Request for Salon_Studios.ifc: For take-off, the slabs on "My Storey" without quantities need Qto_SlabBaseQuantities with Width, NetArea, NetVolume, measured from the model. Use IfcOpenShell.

First a look at what the model holds.

```python
import ifcopenshell
import ifcopenshell.util.element
import ifcopenshell.util.unit

model = ifcopenshell.open("Salon_Studios.ifc")
print(model.schema)
for unit_type in ("LENGTHUNIT", "AREAUNIT", "VOLUMEUNIT"):
    print(unit_type, ifcopenshell.util.unit.calculate_unit_scale(model, unit_type))
storey = next(s for s in model.by_type("IfcBuildingStorey") if s.Name == "My Storey")
slabs = [e for e in ifcopenshell.util.element.get_decomposition(storey) if e.is_a("IfcSlab")]
for e in sorted(slabs, key=lambda e: e.id()):
    print(e.id(), e.is_a(), e.Name, list(ifcopenshell.util.element.get_psets(e, qtos_only=True)), sep=" | ")
```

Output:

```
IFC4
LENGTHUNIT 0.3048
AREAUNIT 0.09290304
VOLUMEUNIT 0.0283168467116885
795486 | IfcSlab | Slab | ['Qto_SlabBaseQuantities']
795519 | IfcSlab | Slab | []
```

```python
import ifcopenshell
import ifcopenshell.api.pset
import ifcopenshell.geom
import ifcopenshell.util.element
import ifcopenshell.util.shape
import ifcopenshell.util.unit

model = ifcopenshell.open("Salon_Studios.ifc")
unit_scale = ifcopenshell.util.unit.calculate_unit_scale(model)
area_scale = ifcopenshell.util.unit.calculate_unit_scale(model, "AREAUNIT")
volume_scale = ifcopenshell.util.unit.calculate_unit_scale(model, "VOLUMEUNIT")
settings = ifcopenshell.geom.settings()

storey = next(s for s in model.by_type("IfcBuildingStorey") if s.Name == "My Storey")
slabs = [e for e in ifcopenshell.util.element.get_decomposition(storey) if e.is_a("IfcSlab")]

for e in sorted(slabs, key=lambda e: e.id()):
    if ifcopenshell.util.element.get_psets(e, qtos_only=True, should_inherit=False):
        continue
    # Geometry comes back in metres, in the element's own axes.
    shape = ifcopenshell.geom.create_shape(settings, e)
    values = {
        "Width": ifcopenshell.util.shape.get_z(shape.geometry) / unit_scale,
        "NetArea": ifcopenshell.util.shape.get_footprint_area(shape.geometry) / area_scale,
        "NetVolume": ifcopenshell.util.shape.get_volume(shape.geometry) / volume_scale,
    }
    qto = ifcopenshell.api.pset.add_qto(model, product=e, name="Qto_SlabBaseQuantities")
    ifcopenshell.api.pset.edit_qto(model, qto=qto, properties=values)
    print(e.id(), {k: round(v, 3) for k, v in values.items()})

model.write("Salon_Studios_rev.ifc")
```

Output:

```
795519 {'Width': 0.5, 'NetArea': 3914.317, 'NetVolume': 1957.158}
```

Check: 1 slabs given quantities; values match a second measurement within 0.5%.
